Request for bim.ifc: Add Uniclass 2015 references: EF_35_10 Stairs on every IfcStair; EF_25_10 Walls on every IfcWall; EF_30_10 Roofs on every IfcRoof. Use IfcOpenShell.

First a look at what the model holds.

```python
import ifcopenshell

model = ifcopenshell.open("bim.ifc")
print(model.schema)
print("classifications:", [c.Name for c in model.by_type("IfcClassification")])
for ifc_class in ("IfcDoor", "IfcRoof", "IfcStair", "IfcWall", "IfcWindow"):
    print(ifc_class, len(model.by_type(ifc_class)))
```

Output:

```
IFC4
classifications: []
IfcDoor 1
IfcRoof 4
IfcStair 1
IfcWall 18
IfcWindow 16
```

```python
import ifcopenshell
import ifcopenshell.api.classification

model = ifcopenshell.open("bim.ifc")

system = ifcopenshell.api.classification.add_classification(model, classification="Uniclass 2015")

codes = {
    "IfcStair": ("EF_35_10", "Stairs"),
    "IfcWall": ("EF_25_10", "Walls"),
    "IfcRoof": ("EF_30_10", "Roofs"),
}
for ifc_class, (code, name) in codes.items():
    products = model.by_type(ifc_class)
    ifcopenshell.api.classification.add_reference(
        model, products=products, classification=system, identification=code, name=name
    )
    print(code, len(products))

model.write("bim_v2.ifc")
```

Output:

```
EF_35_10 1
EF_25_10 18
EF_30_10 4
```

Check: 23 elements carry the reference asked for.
